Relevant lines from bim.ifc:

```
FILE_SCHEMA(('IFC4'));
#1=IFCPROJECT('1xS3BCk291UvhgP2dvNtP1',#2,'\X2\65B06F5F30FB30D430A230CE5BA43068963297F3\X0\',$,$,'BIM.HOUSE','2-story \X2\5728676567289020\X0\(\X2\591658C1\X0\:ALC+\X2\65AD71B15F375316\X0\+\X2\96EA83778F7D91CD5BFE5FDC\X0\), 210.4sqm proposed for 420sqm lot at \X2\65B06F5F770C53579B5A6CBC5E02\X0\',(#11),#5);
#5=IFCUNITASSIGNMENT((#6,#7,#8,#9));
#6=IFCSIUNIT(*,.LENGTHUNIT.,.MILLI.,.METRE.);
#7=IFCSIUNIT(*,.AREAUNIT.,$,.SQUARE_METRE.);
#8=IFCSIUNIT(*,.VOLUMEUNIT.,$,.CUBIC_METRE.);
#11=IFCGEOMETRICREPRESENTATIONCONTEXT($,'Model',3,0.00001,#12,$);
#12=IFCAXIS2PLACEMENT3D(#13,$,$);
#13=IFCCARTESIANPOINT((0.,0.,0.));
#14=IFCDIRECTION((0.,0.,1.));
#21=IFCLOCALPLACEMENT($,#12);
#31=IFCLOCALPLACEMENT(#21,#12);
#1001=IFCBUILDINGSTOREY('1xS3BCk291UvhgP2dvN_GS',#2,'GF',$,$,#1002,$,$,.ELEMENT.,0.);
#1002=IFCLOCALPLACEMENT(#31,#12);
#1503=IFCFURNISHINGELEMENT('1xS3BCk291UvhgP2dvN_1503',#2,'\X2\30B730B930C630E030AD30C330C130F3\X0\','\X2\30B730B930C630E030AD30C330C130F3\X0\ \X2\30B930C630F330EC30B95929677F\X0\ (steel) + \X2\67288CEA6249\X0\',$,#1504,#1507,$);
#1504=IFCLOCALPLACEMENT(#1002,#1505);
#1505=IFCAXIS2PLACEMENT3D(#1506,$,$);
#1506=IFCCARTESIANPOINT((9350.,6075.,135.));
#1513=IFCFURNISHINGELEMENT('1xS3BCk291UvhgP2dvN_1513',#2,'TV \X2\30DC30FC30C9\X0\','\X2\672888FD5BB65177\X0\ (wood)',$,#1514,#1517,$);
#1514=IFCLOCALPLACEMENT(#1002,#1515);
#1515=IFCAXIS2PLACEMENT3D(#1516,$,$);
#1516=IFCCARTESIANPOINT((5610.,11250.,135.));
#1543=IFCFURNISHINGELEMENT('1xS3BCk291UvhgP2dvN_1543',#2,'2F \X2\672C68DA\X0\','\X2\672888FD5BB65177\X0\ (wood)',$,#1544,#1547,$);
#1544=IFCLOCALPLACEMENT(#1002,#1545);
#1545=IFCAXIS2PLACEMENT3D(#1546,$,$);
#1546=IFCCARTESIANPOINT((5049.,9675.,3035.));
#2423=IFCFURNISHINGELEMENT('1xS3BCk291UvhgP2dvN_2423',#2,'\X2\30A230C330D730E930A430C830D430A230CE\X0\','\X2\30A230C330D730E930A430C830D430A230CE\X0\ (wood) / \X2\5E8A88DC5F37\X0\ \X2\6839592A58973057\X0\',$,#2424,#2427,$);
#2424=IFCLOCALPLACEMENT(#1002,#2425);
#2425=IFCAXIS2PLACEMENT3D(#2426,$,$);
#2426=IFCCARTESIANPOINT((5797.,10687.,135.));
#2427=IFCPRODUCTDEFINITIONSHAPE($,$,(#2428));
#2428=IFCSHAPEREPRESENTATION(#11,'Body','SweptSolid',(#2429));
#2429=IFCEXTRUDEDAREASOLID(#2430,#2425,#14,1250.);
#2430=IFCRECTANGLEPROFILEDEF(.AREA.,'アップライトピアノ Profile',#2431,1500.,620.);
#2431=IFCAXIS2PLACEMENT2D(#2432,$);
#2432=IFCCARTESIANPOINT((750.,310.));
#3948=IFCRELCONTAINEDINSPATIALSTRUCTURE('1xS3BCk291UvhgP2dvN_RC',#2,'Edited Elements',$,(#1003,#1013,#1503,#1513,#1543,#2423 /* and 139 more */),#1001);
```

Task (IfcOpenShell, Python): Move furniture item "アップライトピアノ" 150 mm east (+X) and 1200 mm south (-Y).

```python
import ifcopenshell
import ifcopenshell.api.geometry
import ifcopenshell.util.placement
import ifcopenshell.util.unit

model = ifcopenshell.open("bim.ifc")
unit_scale = ifcopenshell.util.unit.calculate_unit_scale(model)

item = model.by_guid("1xS3BCk291UvhgP2dvN_2423")
matrix = ifcopenshell.util.placement.get_local_placement(item.ObjectPlacement)
matrix[0, 3] += 0.15 / unit_scale
matrix[1, 3] -= 1.2 / unit_scale
ifcopenshell.api.geometry.edit_object_placement(model, product=item, matrix=matrix, is_si=False)

print(ifcopenshell.util.placement.get_local_placement(item.ObjectPlacement).round(3) + 0.0)

model.write("bim_edited.ifc")
```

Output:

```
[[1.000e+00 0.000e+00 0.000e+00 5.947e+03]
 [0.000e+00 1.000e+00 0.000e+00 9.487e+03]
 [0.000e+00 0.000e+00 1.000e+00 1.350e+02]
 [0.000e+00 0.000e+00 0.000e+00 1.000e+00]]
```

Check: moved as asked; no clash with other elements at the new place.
